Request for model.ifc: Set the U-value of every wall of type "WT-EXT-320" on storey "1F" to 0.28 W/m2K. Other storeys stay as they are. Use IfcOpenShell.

First a look at what the model holds.

```python
import ifcopenshell
import ifcopenshell.util.element

model = ifcopenshell.open("model.ifc")
print(model.schema)
storey = next(s for s in model.by_type("IfcBuildingStorey") if s.Name == "1F")
walls = [e for e in ifcopenshell.util.element.get_decomposition(storey) if e.is_a("IfcWall")]
seen = {}
for e in walls:
    element_type = ifcopenshell.util.element.get_type(e)
    key = (element_type.Name if element_type != e and element_type else None, ifcopenshell.util.element.get_pset(e, "Pset_WallCommon", "ThermalTransmittance"))
    seen[key] = seen.get(key, 0) + 1
for (name, value), count in sorted(seen.items(), key=str):
    print(count, "x", name, "|", value)
```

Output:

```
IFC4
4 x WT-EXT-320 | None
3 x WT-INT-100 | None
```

```python
import ifcopenshell
import ifcopenshell.api.pset
import ifcopenshell.util.element

model = ifcopenshell.open("model.ifc")

storey = next(s for s in model.by_type("IfcBuildingStorey") if s.Name == "1F")
walls = [e for e in ifcopenshell.util.element.get_decomposition(storey) if e.is_a("IfcWall")]

count = 0
for e in walls:
    element_type = ifcopenshell.util.element.get_type(e)
    if element_type in (None, e) or element_type.Name != "WT-EXT-320":
        continue
    # add_pset returns the element's existing set when there is one.
    pset = ifcopenshell.api.pset.add_pset(model, product=e, name="Pset_WallCommon")
    ifcopenshell.api.pset.edit_pset(model, pset=pset, properties={"ThermalTransmittance": 0.28})
    count += 1

print(count, "walls updated")

model.write("model_v2.ifc")
```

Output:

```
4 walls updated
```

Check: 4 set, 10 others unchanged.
